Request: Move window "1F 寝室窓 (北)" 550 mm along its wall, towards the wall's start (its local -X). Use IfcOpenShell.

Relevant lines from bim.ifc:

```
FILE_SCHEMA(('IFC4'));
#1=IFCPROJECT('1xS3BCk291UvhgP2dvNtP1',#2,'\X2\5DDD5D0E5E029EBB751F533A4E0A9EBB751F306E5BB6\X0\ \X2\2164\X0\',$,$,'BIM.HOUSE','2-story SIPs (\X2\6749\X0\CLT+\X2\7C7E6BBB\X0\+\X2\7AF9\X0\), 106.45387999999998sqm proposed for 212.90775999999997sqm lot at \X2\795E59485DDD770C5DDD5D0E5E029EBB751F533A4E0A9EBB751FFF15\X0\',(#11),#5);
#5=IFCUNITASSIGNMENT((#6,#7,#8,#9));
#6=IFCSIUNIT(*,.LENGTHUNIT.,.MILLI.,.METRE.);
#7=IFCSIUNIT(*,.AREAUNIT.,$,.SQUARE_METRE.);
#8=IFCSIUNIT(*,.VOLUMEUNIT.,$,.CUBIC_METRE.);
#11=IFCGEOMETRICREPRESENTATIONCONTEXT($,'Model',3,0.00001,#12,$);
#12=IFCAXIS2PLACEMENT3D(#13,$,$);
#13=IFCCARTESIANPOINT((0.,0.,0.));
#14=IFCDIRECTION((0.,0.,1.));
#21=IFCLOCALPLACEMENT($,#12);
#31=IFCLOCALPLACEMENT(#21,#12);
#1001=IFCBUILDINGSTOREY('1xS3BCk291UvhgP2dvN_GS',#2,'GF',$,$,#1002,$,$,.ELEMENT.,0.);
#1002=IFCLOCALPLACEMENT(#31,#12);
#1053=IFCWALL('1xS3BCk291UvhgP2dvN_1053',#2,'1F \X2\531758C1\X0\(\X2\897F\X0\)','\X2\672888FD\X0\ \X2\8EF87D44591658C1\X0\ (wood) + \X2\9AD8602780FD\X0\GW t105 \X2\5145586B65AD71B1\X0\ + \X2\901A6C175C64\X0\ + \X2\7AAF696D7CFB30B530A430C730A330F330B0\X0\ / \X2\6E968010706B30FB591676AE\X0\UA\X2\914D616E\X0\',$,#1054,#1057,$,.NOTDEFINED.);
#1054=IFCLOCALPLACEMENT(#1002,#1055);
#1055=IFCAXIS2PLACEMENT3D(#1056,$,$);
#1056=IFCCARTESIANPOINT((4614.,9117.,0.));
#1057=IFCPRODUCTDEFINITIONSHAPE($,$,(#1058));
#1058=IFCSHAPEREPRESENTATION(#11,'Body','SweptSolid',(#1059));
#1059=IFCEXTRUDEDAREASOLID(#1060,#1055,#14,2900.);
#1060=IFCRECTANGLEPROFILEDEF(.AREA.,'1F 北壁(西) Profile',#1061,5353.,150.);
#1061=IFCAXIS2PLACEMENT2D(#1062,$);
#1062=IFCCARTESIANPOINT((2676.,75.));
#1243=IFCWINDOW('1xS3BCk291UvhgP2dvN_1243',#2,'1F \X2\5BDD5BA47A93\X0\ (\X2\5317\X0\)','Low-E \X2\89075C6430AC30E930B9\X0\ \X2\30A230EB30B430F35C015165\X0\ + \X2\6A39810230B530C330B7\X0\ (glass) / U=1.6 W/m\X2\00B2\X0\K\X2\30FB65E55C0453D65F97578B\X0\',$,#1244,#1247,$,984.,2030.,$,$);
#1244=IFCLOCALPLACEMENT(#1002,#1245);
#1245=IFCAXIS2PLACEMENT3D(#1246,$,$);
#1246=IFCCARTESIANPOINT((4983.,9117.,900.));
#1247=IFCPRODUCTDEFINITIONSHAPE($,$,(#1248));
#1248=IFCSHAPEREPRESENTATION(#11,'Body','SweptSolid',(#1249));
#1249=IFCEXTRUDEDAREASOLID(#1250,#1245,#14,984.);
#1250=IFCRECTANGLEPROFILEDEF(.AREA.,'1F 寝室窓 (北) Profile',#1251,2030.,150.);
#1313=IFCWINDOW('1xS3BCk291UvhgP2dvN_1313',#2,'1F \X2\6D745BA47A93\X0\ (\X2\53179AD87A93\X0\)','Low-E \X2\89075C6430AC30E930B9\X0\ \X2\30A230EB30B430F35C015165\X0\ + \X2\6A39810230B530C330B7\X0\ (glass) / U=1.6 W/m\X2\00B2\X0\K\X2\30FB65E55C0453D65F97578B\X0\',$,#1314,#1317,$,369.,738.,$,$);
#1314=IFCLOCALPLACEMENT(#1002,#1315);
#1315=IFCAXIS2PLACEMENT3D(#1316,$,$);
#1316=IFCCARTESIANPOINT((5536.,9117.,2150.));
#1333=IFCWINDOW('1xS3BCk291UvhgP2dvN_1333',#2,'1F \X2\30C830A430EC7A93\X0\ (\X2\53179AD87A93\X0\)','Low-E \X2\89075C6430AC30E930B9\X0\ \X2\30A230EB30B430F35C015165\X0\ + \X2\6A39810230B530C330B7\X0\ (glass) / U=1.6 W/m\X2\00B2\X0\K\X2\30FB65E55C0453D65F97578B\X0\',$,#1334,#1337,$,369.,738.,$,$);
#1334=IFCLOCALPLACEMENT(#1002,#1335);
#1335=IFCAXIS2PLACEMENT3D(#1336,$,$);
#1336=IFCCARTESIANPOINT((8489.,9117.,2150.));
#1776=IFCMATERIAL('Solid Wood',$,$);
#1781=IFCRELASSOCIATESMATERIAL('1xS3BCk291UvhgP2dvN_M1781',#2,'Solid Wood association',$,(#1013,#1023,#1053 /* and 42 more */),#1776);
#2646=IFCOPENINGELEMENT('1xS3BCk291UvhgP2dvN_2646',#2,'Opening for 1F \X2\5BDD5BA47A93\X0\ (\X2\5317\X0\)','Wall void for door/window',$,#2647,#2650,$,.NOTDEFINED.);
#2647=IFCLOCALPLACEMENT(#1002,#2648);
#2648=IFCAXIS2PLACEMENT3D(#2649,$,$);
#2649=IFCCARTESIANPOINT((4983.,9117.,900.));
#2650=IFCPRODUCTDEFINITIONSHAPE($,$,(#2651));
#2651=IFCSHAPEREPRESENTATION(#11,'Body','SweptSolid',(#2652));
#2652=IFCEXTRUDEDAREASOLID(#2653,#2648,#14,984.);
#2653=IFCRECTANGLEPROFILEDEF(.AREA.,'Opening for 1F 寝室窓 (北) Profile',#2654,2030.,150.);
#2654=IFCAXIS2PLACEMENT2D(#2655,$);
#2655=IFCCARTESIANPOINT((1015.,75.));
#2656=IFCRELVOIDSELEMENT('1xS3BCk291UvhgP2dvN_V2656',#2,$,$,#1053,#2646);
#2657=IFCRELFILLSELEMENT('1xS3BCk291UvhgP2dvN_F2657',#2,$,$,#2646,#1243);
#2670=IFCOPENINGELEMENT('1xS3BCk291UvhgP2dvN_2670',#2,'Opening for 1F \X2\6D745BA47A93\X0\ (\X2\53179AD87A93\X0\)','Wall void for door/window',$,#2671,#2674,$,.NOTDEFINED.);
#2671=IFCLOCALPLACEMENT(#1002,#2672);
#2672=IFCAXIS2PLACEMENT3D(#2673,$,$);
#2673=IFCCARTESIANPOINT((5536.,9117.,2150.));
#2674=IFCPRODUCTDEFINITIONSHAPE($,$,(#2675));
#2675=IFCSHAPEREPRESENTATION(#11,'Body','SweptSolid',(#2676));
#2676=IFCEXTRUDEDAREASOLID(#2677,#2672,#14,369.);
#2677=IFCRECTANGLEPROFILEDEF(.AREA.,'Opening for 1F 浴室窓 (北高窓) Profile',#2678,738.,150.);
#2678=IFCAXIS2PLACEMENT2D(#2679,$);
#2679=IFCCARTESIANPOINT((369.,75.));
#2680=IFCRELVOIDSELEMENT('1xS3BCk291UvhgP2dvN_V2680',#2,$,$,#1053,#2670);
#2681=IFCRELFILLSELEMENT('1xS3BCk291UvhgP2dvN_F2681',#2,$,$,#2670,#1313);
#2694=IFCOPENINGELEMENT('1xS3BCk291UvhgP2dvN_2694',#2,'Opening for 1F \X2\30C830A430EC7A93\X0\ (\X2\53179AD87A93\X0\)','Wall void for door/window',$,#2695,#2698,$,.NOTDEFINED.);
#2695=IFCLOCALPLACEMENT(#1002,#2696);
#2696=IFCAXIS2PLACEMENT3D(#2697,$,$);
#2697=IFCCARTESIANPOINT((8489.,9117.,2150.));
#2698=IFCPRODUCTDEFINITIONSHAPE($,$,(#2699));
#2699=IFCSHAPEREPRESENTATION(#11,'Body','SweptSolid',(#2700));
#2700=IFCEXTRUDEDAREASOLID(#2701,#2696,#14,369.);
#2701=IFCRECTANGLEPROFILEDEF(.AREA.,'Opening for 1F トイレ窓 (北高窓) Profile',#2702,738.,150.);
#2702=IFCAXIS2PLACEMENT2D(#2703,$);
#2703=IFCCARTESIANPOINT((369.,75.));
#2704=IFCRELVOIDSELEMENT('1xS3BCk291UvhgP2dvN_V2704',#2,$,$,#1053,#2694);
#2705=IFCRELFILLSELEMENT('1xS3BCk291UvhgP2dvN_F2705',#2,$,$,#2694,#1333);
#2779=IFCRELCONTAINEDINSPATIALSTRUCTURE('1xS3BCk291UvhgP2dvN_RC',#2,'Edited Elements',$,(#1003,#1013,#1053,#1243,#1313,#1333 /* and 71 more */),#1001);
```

```python
import ifcopenshell
import ifcopenshell.api.geometry
import ifcopenshell.util.placement

model = ifcopenshell.open("bim.ifc")

window = model.by_id(1243)
opening = window.FillsVoids[0].RelatingOpeningElement
wall = opening.VoidsElements[0].RelatingBuildingElement

wall_matrix = ifcopenshell.util.placement.get_local_placement(wall.ObjectPlacement)
shift = wall_matrix[:3, 0] * -550.0
before = ifcopenshell.util.placement.get_local_placement(window.ObjectPlacement)[:3, 3].copy()

# The window is not placed relative to its opening, so move both.
for product in (opening, window):
    matrix = ifcopenshell.util.placement.get_local_placement(product.ObjectPlacement)
    matrix[:3, 3] += shift
    ifcopenshell.api.geometry.edit_object_placement(model, product=product, matrix=matrix, is_si=False)

after = ifcopenshell.util.placement.get_local_placement(window.ObjectPlacement)[:3, 3]
print("window moved by", (after - before).round(3) + 0.0)

model.write("bim-out.ifc")
```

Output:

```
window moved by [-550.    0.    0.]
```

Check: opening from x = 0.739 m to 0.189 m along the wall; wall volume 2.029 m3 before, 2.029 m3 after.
